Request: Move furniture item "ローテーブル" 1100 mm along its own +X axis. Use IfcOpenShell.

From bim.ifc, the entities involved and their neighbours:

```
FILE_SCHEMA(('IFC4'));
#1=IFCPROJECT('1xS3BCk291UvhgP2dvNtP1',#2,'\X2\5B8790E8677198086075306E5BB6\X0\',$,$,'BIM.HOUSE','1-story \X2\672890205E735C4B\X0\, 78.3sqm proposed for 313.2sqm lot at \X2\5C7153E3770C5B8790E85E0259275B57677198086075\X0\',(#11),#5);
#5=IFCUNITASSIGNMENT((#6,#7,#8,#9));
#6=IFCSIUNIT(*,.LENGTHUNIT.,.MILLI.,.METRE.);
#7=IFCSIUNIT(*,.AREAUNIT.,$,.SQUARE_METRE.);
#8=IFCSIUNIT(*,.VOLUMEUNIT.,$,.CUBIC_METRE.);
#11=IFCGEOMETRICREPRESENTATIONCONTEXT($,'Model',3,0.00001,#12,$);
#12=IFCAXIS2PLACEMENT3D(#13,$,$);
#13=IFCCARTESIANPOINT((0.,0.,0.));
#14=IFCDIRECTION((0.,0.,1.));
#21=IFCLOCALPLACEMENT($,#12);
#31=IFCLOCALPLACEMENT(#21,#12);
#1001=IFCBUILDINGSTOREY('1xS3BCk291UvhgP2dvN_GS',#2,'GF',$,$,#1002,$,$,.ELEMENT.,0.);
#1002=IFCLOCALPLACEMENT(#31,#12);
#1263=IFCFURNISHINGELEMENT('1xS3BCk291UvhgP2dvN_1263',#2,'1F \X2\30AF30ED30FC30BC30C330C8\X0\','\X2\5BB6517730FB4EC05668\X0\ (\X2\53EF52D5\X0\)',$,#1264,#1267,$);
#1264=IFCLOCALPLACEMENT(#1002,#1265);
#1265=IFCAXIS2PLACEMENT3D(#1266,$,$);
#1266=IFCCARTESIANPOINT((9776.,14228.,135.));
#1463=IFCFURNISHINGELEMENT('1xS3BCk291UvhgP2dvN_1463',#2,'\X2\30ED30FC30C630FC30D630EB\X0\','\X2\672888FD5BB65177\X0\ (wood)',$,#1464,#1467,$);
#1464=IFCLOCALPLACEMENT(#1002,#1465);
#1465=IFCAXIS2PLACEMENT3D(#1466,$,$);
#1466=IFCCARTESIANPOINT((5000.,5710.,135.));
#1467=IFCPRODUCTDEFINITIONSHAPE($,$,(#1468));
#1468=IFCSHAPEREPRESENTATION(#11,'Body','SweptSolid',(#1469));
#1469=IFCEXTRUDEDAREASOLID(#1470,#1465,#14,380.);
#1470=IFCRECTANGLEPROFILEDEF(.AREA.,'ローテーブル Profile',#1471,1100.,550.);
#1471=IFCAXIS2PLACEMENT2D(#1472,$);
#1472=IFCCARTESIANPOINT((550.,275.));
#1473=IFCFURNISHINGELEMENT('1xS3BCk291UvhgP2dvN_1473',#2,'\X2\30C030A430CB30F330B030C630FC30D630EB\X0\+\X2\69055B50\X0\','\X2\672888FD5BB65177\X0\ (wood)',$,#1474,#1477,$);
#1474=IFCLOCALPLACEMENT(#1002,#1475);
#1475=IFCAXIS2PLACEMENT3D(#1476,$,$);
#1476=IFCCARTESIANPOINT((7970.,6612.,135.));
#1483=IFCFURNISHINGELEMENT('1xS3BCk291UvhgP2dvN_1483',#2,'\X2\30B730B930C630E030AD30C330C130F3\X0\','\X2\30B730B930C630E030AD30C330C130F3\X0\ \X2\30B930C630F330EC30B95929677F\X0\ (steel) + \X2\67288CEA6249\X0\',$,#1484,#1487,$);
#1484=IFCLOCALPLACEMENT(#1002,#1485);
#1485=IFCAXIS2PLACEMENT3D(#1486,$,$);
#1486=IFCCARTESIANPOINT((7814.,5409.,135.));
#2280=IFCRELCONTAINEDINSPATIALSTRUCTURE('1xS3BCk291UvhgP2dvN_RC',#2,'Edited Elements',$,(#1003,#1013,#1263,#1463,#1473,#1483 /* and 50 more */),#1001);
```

```python
import ifcopenshell
import ifcopenshell.api.geometry
import ifcopenshell.util.placement

model = ifcopenshell.open("bim.ifc")

item = model.by_guid("1xS3BCk291UvhgP2dvN_1463")
matrix = ifcopenshell.util.placement.get_local_placement(item.ObjectPlacement)
matrix[:3, 3] += matrix[:3, 0] * 1100.0
ifcopenshell.api.geometry.edit_object_placement(model, product=item, matrix=matrix, is_si=False)

print(ifcopenshell.util.placement.get_local_placement(item.ObjectPlacement).round(3) + 0.0)

model.write("bim_v2.ifc")
```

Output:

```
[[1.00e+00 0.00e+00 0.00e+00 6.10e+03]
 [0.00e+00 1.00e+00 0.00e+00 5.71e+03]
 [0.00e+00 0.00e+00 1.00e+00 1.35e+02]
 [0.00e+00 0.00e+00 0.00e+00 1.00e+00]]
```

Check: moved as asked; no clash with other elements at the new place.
